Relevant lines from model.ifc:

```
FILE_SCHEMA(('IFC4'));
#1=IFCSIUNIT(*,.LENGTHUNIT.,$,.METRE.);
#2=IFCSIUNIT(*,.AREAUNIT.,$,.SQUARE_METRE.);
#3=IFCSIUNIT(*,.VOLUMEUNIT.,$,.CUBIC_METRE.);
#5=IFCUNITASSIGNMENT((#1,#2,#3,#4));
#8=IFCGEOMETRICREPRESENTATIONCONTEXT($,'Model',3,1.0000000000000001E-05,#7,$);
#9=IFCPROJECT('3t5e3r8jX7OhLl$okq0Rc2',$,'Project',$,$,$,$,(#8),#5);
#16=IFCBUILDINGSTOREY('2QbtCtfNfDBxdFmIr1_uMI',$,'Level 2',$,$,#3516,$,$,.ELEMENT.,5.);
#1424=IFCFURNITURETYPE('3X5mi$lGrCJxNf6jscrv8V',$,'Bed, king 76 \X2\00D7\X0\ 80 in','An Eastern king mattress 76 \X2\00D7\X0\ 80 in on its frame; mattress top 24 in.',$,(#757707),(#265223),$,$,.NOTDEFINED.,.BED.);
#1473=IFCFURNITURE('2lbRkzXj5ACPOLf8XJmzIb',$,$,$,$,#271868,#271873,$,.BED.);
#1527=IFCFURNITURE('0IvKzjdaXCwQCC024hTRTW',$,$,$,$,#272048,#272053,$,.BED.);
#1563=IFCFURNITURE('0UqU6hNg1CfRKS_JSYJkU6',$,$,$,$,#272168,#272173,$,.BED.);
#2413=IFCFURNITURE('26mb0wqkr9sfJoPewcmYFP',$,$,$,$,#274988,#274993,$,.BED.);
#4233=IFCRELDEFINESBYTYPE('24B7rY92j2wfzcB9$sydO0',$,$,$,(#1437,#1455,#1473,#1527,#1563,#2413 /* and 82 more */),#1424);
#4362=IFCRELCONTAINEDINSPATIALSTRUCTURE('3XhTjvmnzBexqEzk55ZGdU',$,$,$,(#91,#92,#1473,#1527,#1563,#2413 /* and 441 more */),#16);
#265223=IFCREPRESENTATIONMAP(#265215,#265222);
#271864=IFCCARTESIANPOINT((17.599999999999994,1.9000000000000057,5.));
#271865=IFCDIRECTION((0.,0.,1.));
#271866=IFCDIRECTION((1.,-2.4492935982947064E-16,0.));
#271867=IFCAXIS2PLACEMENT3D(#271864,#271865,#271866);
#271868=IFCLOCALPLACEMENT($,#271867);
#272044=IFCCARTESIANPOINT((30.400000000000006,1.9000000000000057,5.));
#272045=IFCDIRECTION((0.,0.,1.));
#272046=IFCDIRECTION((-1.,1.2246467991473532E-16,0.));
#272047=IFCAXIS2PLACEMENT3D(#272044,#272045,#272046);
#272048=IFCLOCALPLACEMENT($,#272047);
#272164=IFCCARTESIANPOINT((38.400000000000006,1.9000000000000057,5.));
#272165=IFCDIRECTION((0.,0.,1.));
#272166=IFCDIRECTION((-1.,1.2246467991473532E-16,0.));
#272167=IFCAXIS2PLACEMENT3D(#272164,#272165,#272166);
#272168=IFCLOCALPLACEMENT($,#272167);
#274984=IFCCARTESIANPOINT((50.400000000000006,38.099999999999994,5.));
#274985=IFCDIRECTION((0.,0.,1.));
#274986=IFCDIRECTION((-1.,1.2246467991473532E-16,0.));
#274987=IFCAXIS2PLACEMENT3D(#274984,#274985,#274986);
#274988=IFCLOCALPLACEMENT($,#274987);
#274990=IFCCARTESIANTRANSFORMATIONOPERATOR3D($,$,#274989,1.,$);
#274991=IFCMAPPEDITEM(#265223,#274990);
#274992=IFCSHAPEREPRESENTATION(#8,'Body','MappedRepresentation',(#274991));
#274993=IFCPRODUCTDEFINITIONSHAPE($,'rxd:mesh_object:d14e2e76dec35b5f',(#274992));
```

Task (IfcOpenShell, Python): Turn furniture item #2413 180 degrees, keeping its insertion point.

```python
import ifcopenshell
import ifcopenshell.api.geometry
import ifcopenshell.util.placement

model = ifcopenshell.open("model.ifc")

item = model.by_id(2413)
matrix = ifcopenshell.util.placement.get_local_placement(item.ObjectPlacement)
matrix = matrix @ ifcopenshell.util.placement.rotation(180, "Z")
ifcopenshell.api.geometry.edit_object_placement(model, product=item, matrix=matrix, is_si=False)

print(ifcopenshell.util.placement.get_local_placement(item.ObjectPlacement).round(3) + 0.0)

model.write("model_edited.ifc")
```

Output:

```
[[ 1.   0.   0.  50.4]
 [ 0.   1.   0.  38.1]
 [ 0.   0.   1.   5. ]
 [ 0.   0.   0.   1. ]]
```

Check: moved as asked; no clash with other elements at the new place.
